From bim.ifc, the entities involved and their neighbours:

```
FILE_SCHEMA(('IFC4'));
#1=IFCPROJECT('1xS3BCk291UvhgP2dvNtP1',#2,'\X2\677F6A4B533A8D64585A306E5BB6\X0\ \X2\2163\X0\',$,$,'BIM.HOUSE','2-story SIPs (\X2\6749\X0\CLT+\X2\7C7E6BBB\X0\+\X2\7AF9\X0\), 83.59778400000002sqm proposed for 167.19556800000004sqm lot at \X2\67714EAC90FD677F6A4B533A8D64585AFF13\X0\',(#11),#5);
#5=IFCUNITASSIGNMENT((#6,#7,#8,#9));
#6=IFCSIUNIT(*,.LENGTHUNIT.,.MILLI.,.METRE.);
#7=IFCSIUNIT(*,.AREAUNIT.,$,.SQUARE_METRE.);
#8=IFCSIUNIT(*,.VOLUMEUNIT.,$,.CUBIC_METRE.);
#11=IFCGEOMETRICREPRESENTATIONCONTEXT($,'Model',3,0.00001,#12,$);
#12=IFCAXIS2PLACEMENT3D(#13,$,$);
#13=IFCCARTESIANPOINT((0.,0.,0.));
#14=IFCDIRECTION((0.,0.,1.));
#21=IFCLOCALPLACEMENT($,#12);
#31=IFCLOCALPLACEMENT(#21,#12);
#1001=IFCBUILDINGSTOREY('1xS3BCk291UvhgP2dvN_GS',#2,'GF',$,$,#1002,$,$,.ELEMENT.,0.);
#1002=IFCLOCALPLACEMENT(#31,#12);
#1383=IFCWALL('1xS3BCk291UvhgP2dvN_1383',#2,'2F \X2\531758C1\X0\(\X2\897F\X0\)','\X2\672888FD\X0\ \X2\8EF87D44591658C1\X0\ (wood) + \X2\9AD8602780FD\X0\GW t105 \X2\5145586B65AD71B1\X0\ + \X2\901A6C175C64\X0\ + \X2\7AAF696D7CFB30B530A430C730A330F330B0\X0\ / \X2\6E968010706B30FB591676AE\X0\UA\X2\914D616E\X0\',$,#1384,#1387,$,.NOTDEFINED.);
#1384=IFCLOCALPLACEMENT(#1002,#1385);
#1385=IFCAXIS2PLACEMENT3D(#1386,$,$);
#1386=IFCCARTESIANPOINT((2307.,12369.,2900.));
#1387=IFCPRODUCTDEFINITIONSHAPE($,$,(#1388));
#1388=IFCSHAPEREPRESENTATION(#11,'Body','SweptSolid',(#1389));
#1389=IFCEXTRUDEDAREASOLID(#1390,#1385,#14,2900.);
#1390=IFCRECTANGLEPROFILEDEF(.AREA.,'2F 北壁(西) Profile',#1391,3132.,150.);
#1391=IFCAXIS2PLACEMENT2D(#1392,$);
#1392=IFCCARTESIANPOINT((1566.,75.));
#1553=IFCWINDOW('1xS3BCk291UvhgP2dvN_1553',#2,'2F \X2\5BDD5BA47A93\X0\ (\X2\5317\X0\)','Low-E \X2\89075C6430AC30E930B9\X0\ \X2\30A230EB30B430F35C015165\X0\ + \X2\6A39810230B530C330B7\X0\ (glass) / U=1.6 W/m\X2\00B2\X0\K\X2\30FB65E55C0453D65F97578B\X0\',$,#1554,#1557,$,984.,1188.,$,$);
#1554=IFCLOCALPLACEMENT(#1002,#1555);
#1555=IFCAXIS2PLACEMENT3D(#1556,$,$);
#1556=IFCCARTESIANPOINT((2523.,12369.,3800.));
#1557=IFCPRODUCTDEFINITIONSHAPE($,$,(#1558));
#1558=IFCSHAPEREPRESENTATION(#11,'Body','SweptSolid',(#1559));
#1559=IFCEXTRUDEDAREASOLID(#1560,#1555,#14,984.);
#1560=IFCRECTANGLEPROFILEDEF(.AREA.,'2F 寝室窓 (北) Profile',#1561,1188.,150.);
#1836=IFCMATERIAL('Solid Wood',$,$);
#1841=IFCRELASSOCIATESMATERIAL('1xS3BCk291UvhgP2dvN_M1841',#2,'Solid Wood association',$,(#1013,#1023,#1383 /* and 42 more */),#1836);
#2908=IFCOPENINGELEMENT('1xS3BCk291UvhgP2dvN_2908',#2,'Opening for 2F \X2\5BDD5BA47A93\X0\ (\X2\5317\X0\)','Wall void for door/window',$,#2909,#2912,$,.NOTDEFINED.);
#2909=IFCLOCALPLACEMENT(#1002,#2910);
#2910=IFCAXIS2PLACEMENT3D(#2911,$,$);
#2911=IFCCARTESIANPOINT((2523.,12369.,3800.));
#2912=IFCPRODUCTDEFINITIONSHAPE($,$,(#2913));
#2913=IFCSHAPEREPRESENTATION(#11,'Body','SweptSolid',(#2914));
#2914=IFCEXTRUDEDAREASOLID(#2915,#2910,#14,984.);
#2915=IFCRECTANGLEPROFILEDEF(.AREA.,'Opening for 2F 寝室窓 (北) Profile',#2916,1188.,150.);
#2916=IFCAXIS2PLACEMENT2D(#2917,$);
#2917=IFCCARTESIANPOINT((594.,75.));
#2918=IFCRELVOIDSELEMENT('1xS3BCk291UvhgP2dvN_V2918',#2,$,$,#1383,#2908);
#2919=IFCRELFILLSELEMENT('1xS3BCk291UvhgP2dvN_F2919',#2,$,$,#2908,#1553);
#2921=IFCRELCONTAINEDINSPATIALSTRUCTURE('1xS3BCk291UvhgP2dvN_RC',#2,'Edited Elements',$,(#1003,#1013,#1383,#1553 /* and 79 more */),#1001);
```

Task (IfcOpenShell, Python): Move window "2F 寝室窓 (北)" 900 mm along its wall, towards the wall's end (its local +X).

```python
import ifcopenshell
import ifcopenshell.api.geometry
import ifcopenshell.util.placement
import ifcopenshell.util.unit

model = ifcopenshell.open("bim.ifc")
unit_scale = ifcopenshell.util.unit.calculate_unit_scale(model)

window = model.by_id(1553)
opening = window.FillsVoids[0].RelatingOpeningElement
wall = opening.VoidsElements[0].RelatingBuildingElement

wall_matrix = ifcopenshell.util.placement.get_local_placement(wall.ObjectPlacement)
shift = wall_matrix[:3, 0] * 0.9 / unit_scale
before = ifcopenshell.util.placement.get_local_placement(window.ObjectPlacement)[:3, 3].copy()

# The window is not placed relative to its opening, so move both.
for product in (opening, window):
    matrix = ifcopenshell.util.placement.get_local_placement(product.ObjectPlacement)
    matrix[:3, 3] += shift
    ifcopenshell.api.geometry.edit_object_placement(model, product=product, matrix=matrix, is_si=False)

after = ifcopenshell.util.placement.get_local_placement(window.ObjectPlacement)[:3, 3]
print("window moved by", (after - before).round(3) + 0.0)

model.write("bim-out.ifc")
```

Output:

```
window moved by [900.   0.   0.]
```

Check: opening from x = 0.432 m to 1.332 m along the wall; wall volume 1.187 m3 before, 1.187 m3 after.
